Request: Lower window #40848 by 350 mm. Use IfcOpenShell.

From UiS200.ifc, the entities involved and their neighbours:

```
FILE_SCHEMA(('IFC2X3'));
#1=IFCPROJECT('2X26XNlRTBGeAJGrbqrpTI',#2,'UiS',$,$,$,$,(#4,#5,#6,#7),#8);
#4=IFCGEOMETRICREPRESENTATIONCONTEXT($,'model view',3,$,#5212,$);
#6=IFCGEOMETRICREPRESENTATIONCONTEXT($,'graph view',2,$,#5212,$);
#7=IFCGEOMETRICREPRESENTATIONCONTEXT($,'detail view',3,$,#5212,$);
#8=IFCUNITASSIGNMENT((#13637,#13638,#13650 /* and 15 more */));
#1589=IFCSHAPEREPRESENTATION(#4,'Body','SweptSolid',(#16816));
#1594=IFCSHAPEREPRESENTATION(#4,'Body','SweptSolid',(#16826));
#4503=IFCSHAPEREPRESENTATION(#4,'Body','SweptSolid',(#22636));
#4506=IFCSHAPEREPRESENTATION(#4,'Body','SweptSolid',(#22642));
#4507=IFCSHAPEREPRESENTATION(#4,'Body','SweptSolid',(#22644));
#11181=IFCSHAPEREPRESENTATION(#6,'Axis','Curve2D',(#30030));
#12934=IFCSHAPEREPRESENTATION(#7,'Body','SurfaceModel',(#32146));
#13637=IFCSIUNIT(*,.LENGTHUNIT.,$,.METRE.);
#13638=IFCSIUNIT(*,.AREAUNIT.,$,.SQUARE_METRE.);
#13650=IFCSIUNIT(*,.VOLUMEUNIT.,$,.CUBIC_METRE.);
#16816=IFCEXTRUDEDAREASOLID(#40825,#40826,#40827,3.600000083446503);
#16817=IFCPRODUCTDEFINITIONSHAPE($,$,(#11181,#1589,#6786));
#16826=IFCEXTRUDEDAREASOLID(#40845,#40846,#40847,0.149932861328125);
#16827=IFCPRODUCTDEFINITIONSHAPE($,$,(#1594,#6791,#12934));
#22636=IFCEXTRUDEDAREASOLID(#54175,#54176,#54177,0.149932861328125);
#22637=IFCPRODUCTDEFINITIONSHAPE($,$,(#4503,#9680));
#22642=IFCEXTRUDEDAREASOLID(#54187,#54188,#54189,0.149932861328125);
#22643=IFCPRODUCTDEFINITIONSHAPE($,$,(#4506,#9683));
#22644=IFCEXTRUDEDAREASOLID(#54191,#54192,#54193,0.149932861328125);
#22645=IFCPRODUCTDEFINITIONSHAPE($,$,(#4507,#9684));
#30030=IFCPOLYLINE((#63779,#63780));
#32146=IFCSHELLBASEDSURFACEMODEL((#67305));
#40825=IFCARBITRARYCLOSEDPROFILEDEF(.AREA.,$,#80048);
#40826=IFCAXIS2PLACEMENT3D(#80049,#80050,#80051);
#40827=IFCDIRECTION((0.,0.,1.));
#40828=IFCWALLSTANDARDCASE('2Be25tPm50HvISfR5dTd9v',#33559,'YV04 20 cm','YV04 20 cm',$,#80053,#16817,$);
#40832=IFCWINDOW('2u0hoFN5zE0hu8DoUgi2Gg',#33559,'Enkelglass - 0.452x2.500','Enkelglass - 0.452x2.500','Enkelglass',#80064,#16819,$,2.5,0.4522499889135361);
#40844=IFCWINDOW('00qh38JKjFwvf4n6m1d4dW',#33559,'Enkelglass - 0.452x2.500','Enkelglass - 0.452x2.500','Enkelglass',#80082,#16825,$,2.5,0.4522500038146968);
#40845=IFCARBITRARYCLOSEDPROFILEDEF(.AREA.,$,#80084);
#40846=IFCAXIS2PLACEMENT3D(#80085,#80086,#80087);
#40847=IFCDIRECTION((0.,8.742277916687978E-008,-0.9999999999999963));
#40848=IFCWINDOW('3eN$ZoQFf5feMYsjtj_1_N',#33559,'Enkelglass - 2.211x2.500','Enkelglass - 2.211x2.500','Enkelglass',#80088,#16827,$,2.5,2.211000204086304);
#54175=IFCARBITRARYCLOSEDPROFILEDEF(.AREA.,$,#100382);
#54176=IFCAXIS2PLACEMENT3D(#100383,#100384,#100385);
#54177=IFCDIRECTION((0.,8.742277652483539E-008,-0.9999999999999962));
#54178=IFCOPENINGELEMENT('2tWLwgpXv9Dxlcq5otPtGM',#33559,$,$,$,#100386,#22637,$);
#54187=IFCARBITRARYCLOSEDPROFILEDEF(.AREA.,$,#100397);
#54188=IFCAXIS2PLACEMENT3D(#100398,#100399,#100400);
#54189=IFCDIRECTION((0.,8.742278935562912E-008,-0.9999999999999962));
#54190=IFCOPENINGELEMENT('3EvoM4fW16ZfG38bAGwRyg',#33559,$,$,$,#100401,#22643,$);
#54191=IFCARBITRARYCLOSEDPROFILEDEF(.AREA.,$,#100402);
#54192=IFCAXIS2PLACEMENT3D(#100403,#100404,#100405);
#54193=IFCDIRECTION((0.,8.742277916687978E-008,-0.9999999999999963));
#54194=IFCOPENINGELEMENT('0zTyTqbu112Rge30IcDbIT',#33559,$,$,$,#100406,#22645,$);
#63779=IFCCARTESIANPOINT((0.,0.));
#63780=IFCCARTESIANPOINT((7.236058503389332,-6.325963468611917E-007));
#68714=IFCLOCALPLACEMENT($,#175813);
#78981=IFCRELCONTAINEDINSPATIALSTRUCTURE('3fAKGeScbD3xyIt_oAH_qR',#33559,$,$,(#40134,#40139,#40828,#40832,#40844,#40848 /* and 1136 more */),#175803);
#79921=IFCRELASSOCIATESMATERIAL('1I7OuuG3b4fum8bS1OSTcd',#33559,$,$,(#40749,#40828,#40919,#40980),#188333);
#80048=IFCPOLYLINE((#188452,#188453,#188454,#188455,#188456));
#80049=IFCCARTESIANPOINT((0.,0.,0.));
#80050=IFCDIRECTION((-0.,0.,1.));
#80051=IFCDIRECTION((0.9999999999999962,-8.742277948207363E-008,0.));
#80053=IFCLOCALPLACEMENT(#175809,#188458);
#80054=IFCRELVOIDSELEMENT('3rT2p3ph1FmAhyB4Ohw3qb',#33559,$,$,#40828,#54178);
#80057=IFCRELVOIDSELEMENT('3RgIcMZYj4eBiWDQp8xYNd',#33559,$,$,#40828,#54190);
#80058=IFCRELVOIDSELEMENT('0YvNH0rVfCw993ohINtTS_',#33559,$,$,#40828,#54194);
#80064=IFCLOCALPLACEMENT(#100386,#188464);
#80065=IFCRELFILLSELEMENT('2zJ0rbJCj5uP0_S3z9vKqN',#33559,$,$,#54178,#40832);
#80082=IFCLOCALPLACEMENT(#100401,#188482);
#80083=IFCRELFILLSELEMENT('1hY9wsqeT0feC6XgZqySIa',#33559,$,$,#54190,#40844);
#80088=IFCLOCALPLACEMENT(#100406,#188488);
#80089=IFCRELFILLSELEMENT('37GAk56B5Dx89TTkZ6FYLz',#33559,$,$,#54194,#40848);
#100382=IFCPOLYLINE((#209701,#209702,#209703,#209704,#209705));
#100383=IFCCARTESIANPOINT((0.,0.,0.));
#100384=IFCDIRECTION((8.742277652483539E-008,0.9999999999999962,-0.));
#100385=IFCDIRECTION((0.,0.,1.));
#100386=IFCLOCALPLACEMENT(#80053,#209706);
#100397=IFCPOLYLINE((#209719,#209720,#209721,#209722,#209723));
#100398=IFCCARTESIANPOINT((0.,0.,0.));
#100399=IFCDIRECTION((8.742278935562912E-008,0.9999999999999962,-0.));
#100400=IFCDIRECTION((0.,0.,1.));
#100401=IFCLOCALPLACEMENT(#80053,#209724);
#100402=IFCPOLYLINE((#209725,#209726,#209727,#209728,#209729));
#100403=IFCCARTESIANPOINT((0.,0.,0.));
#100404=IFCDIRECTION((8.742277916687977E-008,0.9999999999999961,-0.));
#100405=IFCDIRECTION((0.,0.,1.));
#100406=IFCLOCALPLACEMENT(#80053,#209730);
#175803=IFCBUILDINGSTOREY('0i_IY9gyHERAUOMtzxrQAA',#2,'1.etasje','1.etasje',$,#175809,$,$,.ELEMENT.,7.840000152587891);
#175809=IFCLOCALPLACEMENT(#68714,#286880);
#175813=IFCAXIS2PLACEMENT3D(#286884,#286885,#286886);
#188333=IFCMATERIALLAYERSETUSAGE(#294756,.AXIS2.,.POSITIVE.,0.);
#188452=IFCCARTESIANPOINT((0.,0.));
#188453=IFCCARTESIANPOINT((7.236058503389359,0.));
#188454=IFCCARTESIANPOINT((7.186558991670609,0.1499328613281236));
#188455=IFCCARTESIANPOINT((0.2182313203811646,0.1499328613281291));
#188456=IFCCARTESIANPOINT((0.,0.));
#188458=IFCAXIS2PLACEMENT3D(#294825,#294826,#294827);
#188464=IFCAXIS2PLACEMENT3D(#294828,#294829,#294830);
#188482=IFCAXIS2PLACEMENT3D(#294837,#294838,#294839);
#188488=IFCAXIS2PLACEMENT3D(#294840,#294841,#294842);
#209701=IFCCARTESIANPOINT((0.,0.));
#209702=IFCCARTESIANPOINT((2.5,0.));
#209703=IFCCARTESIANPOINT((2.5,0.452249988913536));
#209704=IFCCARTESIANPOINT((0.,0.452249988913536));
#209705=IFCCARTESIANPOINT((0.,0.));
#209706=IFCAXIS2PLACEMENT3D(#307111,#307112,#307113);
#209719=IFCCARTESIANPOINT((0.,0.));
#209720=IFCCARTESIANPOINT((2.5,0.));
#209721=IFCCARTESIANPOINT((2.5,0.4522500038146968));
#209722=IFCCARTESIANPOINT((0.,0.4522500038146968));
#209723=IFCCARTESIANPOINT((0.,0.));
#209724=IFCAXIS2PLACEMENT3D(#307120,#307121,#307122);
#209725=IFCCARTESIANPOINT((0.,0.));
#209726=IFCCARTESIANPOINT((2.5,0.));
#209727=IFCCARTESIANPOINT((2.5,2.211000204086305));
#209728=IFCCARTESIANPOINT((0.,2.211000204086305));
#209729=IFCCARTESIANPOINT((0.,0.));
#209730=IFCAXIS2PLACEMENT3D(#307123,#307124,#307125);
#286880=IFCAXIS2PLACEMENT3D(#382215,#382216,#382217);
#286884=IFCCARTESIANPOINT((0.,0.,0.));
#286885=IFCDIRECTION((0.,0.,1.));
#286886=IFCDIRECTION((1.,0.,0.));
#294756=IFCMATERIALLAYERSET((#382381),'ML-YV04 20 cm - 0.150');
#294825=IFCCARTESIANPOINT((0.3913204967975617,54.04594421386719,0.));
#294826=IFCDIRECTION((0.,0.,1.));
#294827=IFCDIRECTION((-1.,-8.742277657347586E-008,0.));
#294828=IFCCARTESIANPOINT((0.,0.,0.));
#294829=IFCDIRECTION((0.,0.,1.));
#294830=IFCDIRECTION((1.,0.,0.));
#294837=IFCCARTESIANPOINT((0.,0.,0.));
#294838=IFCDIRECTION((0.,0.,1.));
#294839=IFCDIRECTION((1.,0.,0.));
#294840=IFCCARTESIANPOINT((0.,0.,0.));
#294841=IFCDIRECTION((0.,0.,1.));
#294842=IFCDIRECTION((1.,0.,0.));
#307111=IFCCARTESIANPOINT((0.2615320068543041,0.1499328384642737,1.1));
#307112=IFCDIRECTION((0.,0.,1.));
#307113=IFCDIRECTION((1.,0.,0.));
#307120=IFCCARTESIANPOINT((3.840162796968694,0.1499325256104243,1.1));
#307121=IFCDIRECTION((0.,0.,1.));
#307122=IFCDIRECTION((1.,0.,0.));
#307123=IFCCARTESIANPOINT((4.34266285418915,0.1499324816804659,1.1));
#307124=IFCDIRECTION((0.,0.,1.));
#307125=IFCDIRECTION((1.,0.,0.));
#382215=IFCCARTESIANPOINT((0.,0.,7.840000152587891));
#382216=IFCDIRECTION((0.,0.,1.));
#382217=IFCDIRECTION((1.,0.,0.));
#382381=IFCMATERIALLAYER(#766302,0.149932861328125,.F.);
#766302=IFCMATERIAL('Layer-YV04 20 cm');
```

```python
import numpy as np
import ifcopenshell
import ifcopenshell.api.geometry
import ifcopenshell.util.placement
import ifcopenshell.util.unit

model = ifcopenshell.open("UiS200.ifc")
unit_scale = ifcopenshell.util.unit.calculate_unit_scale(model)

window = model.by_guid("3eN$ZoQFf5feMYsjtj_1_N")
opening = window.FillsVoids[0].RelatingOpeningElement
dz = -0.35 / unit_scale

shift = np.array([0.0, 0.0, dz])
# The window is placed relative to its opening, so it follows when the opening moves.
matrix = ifcopenshell.util.placement.get_local_placement(opening.ObjectPlacement)
matrix[:3, 3] += shift
ifcopenshell.api.geometry.edit_object_placement(
    model, product=opening, matrix=matrix, is_si=False, should_transform_children=True
)

print(f"moved by {dz * unit_scale:+.3f} m")

model.write("UiS200-out.ifc")
```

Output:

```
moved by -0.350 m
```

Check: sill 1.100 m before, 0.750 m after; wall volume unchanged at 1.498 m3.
